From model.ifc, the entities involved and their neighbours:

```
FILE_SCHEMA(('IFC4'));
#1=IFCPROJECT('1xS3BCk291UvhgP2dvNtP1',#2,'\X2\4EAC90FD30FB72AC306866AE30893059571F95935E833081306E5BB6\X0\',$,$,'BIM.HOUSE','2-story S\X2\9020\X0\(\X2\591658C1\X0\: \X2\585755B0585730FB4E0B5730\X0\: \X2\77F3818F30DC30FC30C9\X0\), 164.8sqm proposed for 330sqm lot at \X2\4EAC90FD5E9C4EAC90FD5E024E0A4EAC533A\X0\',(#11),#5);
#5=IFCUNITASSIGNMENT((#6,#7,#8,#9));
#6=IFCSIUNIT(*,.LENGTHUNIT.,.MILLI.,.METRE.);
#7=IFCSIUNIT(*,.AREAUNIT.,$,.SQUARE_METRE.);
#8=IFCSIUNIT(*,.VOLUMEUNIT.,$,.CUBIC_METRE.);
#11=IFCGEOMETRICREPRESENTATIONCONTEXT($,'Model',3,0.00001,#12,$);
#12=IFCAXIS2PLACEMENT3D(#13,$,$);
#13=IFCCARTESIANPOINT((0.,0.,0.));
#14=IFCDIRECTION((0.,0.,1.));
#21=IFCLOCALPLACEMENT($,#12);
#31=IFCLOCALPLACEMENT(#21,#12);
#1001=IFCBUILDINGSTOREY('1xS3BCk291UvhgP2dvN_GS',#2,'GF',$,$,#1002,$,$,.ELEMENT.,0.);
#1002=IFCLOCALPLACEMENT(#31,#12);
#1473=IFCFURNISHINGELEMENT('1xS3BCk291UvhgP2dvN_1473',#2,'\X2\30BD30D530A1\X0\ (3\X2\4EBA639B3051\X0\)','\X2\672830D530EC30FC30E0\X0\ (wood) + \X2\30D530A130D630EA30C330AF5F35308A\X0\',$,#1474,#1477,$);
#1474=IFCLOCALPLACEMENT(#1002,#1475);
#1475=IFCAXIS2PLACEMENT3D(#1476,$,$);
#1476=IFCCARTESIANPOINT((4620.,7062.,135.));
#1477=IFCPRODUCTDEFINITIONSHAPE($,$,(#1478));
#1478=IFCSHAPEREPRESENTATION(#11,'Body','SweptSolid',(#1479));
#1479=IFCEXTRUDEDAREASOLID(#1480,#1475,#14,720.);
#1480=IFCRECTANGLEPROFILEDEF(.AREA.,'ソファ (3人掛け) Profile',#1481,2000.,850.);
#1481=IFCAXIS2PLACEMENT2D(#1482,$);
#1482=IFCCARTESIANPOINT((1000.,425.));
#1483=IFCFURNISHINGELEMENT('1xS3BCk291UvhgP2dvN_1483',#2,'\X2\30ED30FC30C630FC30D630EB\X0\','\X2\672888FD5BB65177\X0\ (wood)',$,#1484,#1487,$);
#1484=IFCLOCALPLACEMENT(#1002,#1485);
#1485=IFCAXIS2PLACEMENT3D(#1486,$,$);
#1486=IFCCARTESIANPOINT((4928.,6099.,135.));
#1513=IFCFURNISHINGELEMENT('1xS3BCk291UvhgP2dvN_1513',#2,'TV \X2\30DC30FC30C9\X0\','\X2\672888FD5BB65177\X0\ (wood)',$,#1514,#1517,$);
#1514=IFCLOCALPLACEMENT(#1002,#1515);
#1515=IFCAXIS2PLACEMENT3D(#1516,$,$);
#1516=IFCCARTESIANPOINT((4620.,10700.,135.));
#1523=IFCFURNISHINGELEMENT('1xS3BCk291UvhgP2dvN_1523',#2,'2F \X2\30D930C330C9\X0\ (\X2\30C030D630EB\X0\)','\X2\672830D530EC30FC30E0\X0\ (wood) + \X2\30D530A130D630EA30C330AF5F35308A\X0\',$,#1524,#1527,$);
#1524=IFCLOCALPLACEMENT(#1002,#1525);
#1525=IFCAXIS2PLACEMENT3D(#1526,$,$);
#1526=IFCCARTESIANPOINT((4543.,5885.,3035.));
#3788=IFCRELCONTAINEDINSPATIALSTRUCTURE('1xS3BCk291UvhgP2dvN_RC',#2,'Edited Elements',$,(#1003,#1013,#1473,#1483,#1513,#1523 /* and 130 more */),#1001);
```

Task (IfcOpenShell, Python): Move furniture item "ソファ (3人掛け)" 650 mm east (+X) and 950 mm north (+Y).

```python
import ifcopenshell
import ifcopenshell.api.geometry
import ifcopenshell.util.placement
import ifcopenshell.util.unit

model = ifcopenshell.open("model.ifc")
unit_scale = ifcopenshell.util.unit.calculate_unit_scale(model)

item = model.by_id(1473)
matrix = ifcopenshell.util.placement.get_local_placement(item.ObjectPlacement)
matrix[0, 3] += 0.65 / unit_scale
matrix[1, 3] += 0.95 / unit_scale
ifcopenshell.api.geometry.edit_object_placement(model, product=item, matrix=matrix, is_si=False)

print(ifcopenshell.util.placement.get_local_placement(item.ObjectPlacement).round(3) + 0.0)

model.write("model_rev.ifc")
```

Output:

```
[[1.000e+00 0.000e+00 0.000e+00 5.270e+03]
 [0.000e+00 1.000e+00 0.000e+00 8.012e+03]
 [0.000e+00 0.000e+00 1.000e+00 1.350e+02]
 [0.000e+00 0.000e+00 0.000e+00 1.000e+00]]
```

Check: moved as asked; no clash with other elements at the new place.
